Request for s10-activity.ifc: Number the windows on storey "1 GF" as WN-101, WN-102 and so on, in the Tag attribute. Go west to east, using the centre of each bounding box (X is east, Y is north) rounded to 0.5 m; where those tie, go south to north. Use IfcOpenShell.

First a look at what the model holds.

```python
import ifcopenshell
import ifcopenshell.util.element
import ifcopenshell.util.placement

model = ifcopenshell.open("s10-activity.ifc")
print(model.schema)
storey = next(s for s in model.by_type("IfcBuildingStorey") if s.Name == "1 GF")
windows = [e for e in ifcopenshell.util.element.get_decomposition(storey) if e.is_a("IfcWindow")]
for e in sorted(windows, key=lambda e: e.id()):
    origin = ifcopenshell.util.placement.get_local_placement(e.ObjectPlacement)[:3, 3]
    print(e.id(), e.Tag, e.Name, origin.round(2) + 0.0, sep=" | ")
```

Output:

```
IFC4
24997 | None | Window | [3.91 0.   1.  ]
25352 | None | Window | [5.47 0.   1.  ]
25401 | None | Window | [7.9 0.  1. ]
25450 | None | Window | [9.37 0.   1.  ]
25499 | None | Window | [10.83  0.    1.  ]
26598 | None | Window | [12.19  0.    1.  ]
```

```python
import ifcopenshell
import ifcopenshell.geom
import ifcopenshell.util.element
import ifcopenshell.util.shape

model = ifcopenshell.open("s10-activity.ifc")
settings = ifcopenshell.geom.settings()
settings.set("use-world-coords", True)


def centre(element):
    shape = ifcopenshell.geom.create_shape(settings, element)
    return ifcopenshell.util.shape.get_bbox_centroid(shape.geometry)


storey = next(s for s in model.by_type("IfcBuildingStorey") if s.Name == "1 GF")
windows = [e for e in ifcopenshell.util.element.get_decomposition(storey) if e.is_a("IfcWindow")]

# Insertion points can sit at a corner or the storey origin, so sort by the geometry (in metres).
centres = {e: centre(e) for e in windows}
windows.sort(key=lambda e: (round(centres[e][0] / 0.5), centres[e][1]))

for i, e in enumerate(windows, start=1):
    number = f"WN-1{i:02d}"
    e.Tag = number
    print(e.id(), number)

model.write("s10-activity_v2.ifc")
```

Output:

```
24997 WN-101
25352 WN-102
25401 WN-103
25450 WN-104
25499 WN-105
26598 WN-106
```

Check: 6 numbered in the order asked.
